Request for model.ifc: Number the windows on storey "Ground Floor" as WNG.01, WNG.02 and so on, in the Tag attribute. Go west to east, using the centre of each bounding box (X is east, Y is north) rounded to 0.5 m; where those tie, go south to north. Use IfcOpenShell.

First a look at what the model holds.

```python
import ifcopenshell
import ifcopenshell.util.element
import ifcopenshell.util.placement

model = ifcopenshell.open("model.ifc")
print(model.schema)
storey = next(s for s in model.by_type("IfcBuildingStorey") if s.Name == "Ground Floor")
windows = [e for e in ifcopenshell.util.element.get_decomposition(storey) if e.is_a("IfcWindow")]
for e in sorted(windows, key=lambda e: e.id()):
    origin = ifcopenshell.util.placement.get_local_placement(e.ObjectPlacement)[:3, 3]
    print(e.id(), e.Tag, e.Name, origin.round(2) + 0.0, sep=" | ")
```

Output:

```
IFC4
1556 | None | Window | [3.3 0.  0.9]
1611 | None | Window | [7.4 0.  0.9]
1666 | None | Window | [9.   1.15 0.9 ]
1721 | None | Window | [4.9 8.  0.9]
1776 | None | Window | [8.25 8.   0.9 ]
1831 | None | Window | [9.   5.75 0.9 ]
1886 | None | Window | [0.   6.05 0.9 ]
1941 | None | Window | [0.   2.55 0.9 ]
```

```python
import ifcopenshell
import ifcopenshell.geom
import ifcopenshell.util.element
import ifcopenshell.util.shape

model = ifcopenshell.open("model.ifc")
settings = ifcopenshell.geom.settings()
settings.set("use-world-coords", True)


def centre(element):
    shape = ifcopenshell.geom.create_shape(settings, element)
    return ifcopenshell.util.shape.get_bbox_centroid(shape.geometry)


storey = next(s for s in model.by_type("IfcBuildingStorey") if s.Name == "Ground Floor")
windows = [e for e in ifcopenshell.util.element.get_decomposition(storey) if e.is_a("IfcWindow")]

# Insertion points can sit at a corner or the storey origin, so sort by the geometry (in metres).
centres = {e: centre(e) for e in windows}
windows.sort(key=lambda e: (round(centres[e][0] / 0.5), centres[e][1]))

for i, e in enumerate(windows, start=1):
    number = f"WNG.{i:02d}"
    e.Tag = number
    print(e.id(), number)

model.write("model_edited.ifc")
```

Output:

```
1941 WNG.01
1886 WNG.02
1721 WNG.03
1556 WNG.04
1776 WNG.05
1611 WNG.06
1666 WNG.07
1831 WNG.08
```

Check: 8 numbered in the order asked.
